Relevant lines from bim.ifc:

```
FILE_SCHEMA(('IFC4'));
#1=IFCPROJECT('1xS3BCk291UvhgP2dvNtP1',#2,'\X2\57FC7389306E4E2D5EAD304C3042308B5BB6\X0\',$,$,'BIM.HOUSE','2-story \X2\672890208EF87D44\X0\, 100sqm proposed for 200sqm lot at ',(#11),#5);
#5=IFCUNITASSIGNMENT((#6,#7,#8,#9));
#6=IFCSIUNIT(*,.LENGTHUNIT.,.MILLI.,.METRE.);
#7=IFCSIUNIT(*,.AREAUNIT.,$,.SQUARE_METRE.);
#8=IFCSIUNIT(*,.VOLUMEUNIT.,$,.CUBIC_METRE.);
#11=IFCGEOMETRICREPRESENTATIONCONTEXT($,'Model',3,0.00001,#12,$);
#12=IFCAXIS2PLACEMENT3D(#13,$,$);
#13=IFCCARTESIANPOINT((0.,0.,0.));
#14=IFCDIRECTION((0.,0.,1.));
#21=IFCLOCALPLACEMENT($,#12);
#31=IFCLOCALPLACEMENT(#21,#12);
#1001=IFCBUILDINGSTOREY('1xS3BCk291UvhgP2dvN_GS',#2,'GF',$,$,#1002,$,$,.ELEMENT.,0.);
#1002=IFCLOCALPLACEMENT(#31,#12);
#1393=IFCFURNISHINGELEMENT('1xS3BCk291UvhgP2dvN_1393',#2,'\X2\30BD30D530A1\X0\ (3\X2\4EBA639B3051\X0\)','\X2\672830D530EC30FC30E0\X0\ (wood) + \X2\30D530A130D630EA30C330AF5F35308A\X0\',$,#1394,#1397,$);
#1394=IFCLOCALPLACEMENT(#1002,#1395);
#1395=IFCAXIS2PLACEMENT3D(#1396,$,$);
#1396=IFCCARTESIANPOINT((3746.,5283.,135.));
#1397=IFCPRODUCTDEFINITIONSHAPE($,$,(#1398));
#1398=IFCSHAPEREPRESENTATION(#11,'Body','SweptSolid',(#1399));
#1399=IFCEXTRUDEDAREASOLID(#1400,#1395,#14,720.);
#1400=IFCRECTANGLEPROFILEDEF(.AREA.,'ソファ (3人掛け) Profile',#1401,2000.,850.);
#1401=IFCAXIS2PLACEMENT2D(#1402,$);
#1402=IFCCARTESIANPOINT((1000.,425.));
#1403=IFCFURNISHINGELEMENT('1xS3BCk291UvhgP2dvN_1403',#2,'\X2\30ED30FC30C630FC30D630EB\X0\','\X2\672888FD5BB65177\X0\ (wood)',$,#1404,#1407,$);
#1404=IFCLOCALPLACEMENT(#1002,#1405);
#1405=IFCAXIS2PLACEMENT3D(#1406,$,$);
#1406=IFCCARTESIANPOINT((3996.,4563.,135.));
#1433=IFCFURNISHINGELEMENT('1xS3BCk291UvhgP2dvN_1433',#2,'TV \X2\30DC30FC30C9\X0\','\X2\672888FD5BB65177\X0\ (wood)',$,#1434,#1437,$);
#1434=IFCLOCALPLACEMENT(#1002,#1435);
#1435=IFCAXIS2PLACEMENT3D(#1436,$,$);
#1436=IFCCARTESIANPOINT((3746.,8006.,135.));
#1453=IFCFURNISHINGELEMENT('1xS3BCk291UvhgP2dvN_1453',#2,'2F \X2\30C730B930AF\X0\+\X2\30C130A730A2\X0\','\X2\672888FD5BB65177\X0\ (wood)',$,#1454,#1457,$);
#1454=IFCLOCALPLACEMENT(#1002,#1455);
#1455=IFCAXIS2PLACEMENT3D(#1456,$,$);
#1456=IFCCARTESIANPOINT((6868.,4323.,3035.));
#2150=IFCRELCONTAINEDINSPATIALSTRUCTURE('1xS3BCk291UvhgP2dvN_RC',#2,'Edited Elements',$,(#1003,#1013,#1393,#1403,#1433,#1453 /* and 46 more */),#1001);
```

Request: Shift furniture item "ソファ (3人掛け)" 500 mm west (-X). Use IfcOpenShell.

```python
import ifcopenshell
import ifcopenshell.api.geometry
import ifcopenshell.util.placement

model = ifcopenshell.open("bim.ifc")

item = model.by_guid("1xS3BCk291UvhgP2dvN_1393")
matrix = ifcopenshell.util.placement.get_local_placement(item.ObjectPlacement)
matrix[0, 3] -= 500.0
ifcopenshell.api.geometry.edit_object_placement(model, product=item, matrix=matrix, is_si=False)

print(ifcopenshell.util.placement.get_local_placement(item.ObjectPlacement).round(3) + 0.0)

model.write("bim_edited.ifc")
```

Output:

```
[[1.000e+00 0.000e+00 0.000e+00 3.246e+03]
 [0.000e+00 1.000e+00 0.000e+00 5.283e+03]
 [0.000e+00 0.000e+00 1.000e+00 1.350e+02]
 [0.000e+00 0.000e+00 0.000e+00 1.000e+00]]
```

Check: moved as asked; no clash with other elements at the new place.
